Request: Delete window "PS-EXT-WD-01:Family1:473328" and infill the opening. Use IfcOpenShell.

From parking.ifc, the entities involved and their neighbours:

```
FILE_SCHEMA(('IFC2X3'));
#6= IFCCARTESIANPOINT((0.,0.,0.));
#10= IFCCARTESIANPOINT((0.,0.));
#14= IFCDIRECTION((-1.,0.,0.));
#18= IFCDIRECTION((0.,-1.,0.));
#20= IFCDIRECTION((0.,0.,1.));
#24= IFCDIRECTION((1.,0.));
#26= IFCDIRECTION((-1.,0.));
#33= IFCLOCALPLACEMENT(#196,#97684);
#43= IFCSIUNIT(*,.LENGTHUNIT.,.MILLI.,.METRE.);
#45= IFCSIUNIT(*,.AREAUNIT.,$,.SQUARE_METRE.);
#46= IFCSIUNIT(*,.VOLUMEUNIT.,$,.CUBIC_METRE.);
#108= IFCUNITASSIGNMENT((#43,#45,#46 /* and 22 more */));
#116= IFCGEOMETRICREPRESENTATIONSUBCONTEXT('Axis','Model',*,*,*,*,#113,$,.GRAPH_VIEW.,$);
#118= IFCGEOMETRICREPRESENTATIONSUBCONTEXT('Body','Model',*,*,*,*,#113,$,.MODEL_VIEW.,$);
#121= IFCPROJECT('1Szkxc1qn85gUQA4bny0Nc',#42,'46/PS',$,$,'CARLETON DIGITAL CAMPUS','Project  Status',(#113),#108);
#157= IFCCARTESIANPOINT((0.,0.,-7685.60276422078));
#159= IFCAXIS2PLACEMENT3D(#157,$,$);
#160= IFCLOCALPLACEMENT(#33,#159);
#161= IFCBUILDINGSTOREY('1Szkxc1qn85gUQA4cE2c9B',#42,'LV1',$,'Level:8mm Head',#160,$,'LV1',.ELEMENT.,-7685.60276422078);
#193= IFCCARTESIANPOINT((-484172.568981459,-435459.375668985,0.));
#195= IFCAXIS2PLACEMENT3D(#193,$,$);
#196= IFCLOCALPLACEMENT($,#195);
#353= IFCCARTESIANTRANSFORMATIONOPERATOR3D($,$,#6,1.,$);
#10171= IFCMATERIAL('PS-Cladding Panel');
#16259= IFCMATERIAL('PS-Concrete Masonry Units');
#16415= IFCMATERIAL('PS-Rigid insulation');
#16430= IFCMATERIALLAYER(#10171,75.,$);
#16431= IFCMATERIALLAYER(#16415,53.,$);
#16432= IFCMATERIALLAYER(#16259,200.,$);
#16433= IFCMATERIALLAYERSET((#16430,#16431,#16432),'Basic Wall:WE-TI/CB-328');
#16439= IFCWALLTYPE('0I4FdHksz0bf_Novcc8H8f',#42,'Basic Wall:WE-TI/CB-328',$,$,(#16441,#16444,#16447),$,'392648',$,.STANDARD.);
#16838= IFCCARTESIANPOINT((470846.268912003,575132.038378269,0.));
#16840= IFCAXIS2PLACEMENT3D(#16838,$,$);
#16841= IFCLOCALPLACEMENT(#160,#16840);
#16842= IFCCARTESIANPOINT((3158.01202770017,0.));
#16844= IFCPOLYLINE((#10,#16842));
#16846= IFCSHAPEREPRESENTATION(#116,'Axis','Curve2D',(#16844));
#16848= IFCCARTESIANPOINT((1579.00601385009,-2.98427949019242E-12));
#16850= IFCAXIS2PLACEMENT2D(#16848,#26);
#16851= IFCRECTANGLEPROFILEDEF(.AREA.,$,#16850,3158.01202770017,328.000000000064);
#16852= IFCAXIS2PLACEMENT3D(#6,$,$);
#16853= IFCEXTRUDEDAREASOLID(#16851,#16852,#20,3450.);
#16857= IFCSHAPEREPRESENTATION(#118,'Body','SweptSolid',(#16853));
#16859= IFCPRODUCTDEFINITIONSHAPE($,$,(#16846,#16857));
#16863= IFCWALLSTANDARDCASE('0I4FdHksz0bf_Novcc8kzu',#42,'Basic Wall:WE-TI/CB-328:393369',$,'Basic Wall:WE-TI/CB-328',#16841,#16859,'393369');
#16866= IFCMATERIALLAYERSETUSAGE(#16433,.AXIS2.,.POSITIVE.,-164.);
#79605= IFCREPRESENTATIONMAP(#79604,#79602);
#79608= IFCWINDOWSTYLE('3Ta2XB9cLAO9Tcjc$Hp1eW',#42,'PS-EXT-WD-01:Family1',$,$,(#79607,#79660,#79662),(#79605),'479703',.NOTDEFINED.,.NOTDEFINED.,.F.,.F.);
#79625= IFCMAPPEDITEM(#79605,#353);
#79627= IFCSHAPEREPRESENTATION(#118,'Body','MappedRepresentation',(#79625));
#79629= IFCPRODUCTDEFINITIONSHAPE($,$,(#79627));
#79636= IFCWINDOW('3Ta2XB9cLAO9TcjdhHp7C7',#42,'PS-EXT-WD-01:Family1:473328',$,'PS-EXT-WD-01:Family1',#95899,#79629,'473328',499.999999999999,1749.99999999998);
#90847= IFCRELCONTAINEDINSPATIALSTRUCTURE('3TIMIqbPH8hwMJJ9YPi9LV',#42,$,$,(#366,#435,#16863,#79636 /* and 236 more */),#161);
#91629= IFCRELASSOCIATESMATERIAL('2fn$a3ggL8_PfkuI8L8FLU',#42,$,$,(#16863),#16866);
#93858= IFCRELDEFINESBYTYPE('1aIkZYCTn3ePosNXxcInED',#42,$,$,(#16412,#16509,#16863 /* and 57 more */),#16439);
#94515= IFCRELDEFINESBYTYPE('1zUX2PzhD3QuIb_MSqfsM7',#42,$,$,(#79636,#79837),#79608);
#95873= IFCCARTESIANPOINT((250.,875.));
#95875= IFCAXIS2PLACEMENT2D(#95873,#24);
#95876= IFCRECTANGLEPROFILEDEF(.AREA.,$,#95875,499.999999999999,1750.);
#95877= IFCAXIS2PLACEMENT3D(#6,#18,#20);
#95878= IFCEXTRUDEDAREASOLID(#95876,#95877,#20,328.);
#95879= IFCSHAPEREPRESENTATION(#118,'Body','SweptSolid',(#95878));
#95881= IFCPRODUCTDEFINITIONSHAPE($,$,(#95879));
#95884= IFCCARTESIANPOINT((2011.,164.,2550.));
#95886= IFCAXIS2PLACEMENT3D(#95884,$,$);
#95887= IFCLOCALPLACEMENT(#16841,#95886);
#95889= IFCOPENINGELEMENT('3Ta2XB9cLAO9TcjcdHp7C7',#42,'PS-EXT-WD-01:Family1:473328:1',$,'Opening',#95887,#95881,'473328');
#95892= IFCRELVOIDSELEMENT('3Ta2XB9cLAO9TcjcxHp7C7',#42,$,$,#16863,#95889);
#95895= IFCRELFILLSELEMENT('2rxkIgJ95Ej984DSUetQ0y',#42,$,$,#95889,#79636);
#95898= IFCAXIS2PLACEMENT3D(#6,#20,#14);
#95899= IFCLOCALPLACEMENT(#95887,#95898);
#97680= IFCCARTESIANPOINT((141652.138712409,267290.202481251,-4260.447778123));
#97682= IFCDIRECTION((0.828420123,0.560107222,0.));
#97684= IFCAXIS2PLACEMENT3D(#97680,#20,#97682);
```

```python
import ifcopenshell
import ifcopenshell.api.feature
import ifcopenshell.api.root
import ifcopenshell.geom
import ifcopenshell.util.shape

model = ifcopenshell.open("parking.ifc")
settings = ifcopenshell.geom.settings()


def volume(element):
    """Net volume in cubic metres, openings subtracted."""
    shape = ifcopenshell.geom.create_shape(settings, element)
    return ifcopenshell.util.shape.get_volume(shape.geometry)


window = model.by_guid("3Ta2XB9cLAO9TcjdhHp7C7")
opening = window.FillsVoids[0].RelatingOpeningElement
wall = opening.VoidsElements[0].RelatingBuildingElement
before = volume(wall)

ifcopenshell.api.root.remove_product(model, product=window)
ifcopenshell.api.feature.remove_feature(model, feature=opening)

after = volume(wall)

print(f"wall volume {before:.3f} -> {after:.3f} m3")

model.write("parking_updated.ifc")
```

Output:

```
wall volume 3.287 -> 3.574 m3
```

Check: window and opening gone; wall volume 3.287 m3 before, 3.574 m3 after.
